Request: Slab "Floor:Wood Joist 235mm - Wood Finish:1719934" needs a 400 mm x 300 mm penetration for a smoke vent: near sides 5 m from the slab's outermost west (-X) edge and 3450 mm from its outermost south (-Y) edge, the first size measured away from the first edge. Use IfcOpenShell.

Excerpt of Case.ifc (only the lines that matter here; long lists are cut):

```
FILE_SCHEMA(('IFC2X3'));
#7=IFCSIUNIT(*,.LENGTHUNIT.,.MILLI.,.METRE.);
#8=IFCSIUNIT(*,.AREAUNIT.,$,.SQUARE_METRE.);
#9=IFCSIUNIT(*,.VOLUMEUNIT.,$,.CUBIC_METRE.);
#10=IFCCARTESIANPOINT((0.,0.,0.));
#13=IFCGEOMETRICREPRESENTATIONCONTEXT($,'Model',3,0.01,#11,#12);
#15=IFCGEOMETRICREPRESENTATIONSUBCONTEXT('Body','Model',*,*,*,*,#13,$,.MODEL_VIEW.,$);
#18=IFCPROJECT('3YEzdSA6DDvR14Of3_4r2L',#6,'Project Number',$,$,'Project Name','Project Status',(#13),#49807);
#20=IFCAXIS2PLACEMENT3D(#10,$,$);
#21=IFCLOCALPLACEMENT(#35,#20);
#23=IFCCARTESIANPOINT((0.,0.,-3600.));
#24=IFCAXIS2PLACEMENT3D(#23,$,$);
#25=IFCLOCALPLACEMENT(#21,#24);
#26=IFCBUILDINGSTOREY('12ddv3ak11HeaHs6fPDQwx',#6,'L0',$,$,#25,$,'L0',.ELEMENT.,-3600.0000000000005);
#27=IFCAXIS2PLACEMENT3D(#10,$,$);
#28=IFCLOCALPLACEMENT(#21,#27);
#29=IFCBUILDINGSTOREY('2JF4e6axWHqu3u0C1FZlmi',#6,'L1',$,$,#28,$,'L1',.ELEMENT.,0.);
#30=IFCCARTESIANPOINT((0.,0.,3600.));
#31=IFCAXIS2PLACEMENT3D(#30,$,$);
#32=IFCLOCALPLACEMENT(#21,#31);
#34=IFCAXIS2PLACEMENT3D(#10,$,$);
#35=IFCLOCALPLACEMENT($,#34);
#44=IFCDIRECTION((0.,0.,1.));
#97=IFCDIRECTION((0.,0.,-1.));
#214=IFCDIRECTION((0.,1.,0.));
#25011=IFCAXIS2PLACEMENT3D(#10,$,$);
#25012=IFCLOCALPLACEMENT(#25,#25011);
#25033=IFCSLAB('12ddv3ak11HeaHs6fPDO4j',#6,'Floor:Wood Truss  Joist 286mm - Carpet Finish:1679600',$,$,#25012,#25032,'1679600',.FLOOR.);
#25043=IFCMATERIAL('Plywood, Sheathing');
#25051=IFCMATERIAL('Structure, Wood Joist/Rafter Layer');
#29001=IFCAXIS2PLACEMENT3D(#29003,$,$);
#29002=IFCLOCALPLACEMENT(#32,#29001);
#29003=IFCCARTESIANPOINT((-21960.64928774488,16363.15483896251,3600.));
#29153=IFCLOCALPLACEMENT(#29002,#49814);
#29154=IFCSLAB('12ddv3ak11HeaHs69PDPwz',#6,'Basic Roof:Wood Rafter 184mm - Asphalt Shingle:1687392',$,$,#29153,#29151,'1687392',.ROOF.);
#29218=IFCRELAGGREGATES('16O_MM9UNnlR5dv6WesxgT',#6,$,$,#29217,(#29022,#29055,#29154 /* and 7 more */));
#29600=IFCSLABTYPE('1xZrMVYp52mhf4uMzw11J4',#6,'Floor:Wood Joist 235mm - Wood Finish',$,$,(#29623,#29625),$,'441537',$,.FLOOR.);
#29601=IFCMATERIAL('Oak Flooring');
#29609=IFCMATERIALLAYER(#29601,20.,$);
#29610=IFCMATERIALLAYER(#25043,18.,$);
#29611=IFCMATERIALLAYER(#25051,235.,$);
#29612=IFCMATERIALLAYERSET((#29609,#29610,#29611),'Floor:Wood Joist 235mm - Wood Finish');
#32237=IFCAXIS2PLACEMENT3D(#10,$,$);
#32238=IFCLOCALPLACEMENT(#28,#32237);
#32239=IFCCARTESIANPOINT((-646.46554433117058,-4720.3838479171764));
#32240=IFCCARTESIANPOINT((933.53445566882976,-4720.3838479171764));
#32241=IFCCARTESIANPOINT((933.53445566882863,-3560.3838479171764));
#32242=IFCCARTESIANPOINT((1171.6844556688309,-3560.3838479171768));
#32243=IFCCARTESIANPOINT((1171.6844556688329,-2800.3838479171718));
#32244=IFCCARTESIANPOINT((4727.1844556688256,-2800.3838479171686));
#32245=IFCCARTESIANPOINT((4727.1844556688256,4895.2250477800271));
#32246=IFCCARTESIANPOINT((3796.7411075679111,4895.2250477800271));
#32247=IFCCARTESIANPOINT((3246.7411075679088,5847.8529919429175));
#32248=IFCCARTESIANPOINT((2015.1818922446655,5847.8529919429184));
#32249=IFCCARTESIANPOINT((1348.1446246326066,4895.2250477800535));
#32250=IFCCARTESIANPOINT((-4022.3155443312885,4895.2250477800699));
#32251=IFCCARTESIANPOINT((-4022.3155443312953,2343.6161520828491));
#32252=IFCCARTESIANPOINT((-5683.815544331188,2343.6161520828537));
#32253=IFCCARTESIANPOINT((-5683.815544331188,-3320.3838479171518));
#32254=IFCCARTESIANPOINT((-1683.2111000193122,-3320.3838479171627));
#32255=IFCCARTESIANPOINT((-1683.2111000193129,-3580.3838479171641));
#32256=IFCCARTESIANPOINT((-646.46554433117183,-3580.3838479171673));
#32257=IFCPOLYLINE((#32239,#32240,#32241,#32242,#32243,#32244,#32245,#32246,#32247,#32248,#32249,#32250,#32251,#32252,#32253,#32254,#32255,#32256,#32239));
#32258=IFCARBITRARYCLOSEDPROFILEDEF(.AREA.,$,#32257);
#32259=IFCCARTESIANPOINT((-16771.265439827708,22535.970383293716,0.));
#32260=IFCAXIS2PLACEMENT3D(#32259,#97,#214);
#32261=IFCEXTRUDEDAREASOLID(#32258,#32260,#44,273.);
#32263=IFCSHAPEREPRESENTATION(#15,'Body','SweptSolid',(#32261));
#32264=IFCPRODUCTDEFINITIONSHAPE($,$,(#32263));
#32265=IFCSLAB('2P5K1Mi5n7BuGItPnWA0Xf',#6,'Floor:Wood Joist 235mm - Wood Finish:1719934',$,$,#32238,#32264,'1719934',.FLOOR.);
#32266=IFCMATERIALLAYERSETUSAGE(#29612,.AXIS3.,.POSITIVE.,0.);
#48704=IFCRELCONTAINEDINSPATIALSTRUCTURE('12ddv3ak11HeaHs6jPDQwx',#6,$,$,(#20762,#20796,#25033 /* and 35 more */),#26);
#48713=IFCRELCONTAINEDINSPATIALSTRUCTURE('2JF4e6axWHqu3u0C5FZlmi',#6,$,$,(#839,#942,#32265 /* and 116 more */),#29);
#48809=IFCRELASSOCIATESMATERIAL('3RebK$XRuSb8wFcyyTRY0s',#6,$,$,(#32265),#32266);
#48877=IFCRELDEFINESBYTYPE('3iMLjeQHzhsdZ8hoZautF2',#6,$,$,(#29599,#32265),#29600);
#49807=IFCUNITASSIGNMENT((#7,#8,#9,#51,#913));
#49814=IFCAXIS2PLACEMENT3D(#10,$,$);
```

```python
import numpy as np
import ifcopenshell
import ifcopenshell.api.feature
import ifcopenshell.api.geometry
import ifcopenshell.api.root
import ifcopenshell.geom
import ifcopenshell.util.placement
import ifcopenshell.util.representation
import ifcopenshell.util.shape
import ifcopenshell.util.unit

model = ifcopenshell.open("Case.ifc")
unit_scale = ifcopenshell.util.unit.calculate_unit_scale(model)
settings = ifcopenshell.geom.settings()


def volume(element):
    """Net volume in cubic metres, openings subtracted."""
    shape = ifcopenshell.geom.create_shape(settings, element)
    return ifcopenshell.util.shape.get_volume(shape.geometry)


slab = model.by_id(32265)
before = volume(slab)

# Extent in the slab's own axes, in metres. The edges named are its -X and -Y sides.
slab_shape = ifcopenshell.geom.create_shape(settings, slab)
vertices = ifcopenshell.util.shape.get_vertices(slab_shape.geometry)
x_min, y_min, bottom = vertices.min(axis=0)
top = vertices[:, 2].max()

opening = ifcopenshell.api.root.create_entity(model, ifc_class="IfcOpeningElement", name="Smoke vent opening")
context = ifcopenshell.util.representation.get_context(model, "Model", "Body", "MODEL_VIEW")
width, depth = 0.4, 0.3
outline = [(0.0, 0.0), (width, 0.0), (width, depth), (0.0, depth), (0.0, 0.0)]
# Overshoot both faces by 50 mm so the cut is clean.
shape = ifcopenshell.api.geometry.add_slab_representation(
    model, context=context, depth=top - bottom + 0.1, polyline=outline
)
ifcopenshell.api.geometry.assign_representation(model, product=opening, representation=shape)

matrix = ifcopenshell.util.placement.get_local_placement(slab.ObjectPlacement)
matrix[:, 3] = matrix @ np.append(np.array([x_min + 5, y_min + 3.45, bottom - 0.05]) / unit_scale, 1.0)
ifcopenshell.api.geometry.edit_object_placement(model, product=opening, matrix=matrix, is_si=False)
ifcopenshell.api.feature.add_feature(model, feature=opening, element=slab)

after = volume(slab)

print(f"slab volume {before:.3f} -> {after:.3f} m3")

model.write("Case_rev.ifc")
```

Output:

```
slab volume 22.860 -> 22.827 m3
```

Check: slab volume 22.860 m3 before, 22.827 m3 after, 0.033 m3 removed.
